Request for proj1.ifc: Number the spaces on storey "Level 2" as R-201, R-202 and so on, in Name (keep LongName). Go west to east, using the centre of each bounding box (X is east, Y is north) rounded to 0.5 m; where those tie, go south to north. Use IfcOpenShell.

First a look at what the model holds.

```python
import ifcopenshell
import ifcopenshell.util.element
import ifcopenshell.util.placement

model = ifcopenshell.open("proj1.ifc")
print(model.schema)
storey = next(s for s in model.by_type("IfcBuildingStorey") if s.Name == "Level 2")
spaces = [e for e in ifcopenshell.util.element.get_decomposition(storey) if e.is_a("IfcSpace")]
for e in sorted(spaces, key=lambda e: e.id()):
    origin = ifcopenshell.util.placement.get_local_placement(e.ObjectPlacement)[:3, 3]
    print(e.id(), e.Name, e.LongName, origin.round(2) + 0.0, sep=" | ")
```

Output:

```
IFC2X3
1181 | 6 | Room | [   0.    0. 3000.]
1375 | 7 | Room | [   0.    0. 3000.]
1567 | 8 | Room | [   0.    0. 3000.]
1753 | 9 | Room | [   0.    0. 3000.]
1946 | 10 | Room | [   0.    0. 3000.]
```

```python
import ifcopenshell
import ifcopenshell.geom
import ifcopenshell.util.element
import ifcopenshell.util.shape

model = ifcopenshell.open("proj1.ifc")
settings = ifcopenshell.geom.settings()
settings.set("use-world-coords", True)


def centre(element):
    shape = ifcopenshell.geom.create_shape(settings, element)
    return ifcopenshell.util.shape.get_bbox_centroid(shape.geometry)


storey = next(s for s in model.by_type("IfcBuildingStorey") if s.Name == "Level 2")
spaces = [e for e in ifcopenshell.util.element.get_decomposition(storey) if e.is_a("IfcSpace")]

# Insertion points can sit at a corner or the storey origin, so sort by the geometry (in metres).
centres = {e: centre(e) for e in spaces}
spaces.sort(key=lambda e: (round(centres[e][0] / 0.5), centres[e][1]))

for i, e in enumerate(spaces, start=1):
    number = f"R-2{i:02d}"
    e.Name = number
    print(e.id(), number)

model.write("proj1_rev.ifc")
```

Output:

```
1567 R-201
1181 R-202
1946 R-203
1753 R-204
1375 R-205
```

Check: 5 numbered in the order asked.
